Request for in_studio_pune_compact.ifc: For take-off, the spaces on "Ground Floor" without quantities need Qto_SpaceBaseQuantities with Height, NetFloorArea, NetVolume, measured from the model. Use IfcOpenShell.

First a look at what the model holds.

```python
import ifcopenshell
import ifcopenshell.util.element
import ifcopenshell.util.unit

model = ifcopenshell.open("in_studio_pune_compact.ifc")
print(model.schema)
for unit_type in ("LENGTHUNIT", "AREAUNIT", "VOLUMEUNIT"):
    print(unit_type, ifcopenshell.util.unit.calculate_unit_scale(model, unit_type))
storey = next(s for s in model.by_type("IfcBuildingStorey") if s.Name == "Ground Floor")
spaces = [e for e in ifcopenshell.util.element.get_decomposition(storey) if e.is_a("IfcSpace")]
for e in sorted(spaces, key=lambda e: e.id()):
    print(e.id(), e.is_a(), e.Name, list(ifcopenshell.util.element.get_psets(e, qtos_only=True)), sep=" | ")
```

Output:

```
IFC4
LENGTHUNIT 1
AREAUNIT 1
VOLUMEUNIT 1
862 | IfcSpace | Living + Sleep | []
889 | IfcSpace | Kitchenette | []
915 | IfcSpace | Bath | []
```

```python
import ifcopenshell
import ifcopenshell.api.pset
import ifcopenshell.geom
import ifcopenshell.util.element
import ifcopenshell.util.shape
import ifcopenshell.util.unit

model = ifcopenshell.open("in_studio_pune_compact.ifc")
unit_scale = ifcopenshell.util.unit.calculate_unit_scale(model)
area_scale = ifcopenshell.util.unit.calculate_unit_scale(model, "AREAUNIT")
volume_scale = ifcopenshell.util.unit.calculate_unit_scale(model, "VOLUMEUNIT")
settings = ifcopenshell.geom.settings()

storey = next(s for s in model.by_type("IfcBuildingStorey") if s.Name == "Ground Floor")
spaces = [e for e in ifcopenshell.util.element.get_decomposition(storey) if e.is_a("IfcSpace")]

for e in sorted(spaces, key=lambda e: e.id()):
    if ifcopenshell.util.element.get_psets(e, qtos_only=True, should_inherit=False):
        continue
    # Geometry comes back in metres, in the element's own axes.
    shape = ifcopenshell.geom.create_shape(settings, e)
    values = {
        "Height": ifcopenshell.util.shape.get_z(shape.geometry) / unit_scale,
        "NetFloorArea": ifcopenshell.util.shape.get_footprint_area(shape.geometry) / area_scale,
        "NetVolume": ifcopenshell.util.shape.get_volume(shape.geometry) / volume_scale,
    }
    qto = ifcopenshell.api.pset.add_qto(model, product=e, name="Qto_SpaceBaseQuantities")
    ifcopenshell.api.pset.edit_qto(model, qto=qto, properties=values)
    print(e.id(), {k: round(v, 3) for k, v in values.items()})

model.write("in_studio_pune_compact_edited.ifc")
```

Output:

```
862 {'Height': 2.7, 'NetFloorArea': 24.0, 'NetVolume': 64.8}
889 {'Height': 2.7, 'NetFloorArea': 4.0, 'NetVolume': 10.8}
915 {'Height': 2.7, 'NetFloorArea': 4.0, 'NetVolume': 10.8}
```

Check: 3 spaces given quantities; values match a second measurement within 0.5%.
